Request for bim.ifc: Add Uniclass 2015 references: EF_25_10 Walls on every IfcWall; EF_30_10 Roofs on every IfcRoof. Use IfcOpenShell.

First a look at what the model holds.

```python
import ifcopenshell

model = ifcopenshell.open("bim.ifc")
print(model.schema)
print("classifications:", [c.Name for c in model.by_type("IfcClassification")])
for ifc_class in ("IfcDoor", "IfcRoof", "IfcStair", "IfcWall", "IfcWindow"):
    print(ifc_class, len(model.by_type(ifc_class)))
```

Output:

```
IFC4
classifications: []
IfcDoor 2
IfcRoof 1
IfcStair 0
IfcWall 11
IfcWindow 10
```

```python
import ifcopenshell
import ifcopenshell.api.classification

model = ifcopenshell.open("bim.ifc")

system = ifcopenshell.api.classification.add_classification(model, classification="Uniclass 2015")

codes = {
    "IfcWall": ("EF_25_10", "Walls"),
    "IfcRoof": ("EF_30_10", "Roofs"),
}
for ifc_class, (code, name) in codes.items():
    products = model.by_type(ifc_class)
    ifcopenshell.api.classification.add_reference(
        model, products=products, classification=system, identification=code, name=name
    )
    print(code, len(products))

model.write("bim_rev.ifc")
```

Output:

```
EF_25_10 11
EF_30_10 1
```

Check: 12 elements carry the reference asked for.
